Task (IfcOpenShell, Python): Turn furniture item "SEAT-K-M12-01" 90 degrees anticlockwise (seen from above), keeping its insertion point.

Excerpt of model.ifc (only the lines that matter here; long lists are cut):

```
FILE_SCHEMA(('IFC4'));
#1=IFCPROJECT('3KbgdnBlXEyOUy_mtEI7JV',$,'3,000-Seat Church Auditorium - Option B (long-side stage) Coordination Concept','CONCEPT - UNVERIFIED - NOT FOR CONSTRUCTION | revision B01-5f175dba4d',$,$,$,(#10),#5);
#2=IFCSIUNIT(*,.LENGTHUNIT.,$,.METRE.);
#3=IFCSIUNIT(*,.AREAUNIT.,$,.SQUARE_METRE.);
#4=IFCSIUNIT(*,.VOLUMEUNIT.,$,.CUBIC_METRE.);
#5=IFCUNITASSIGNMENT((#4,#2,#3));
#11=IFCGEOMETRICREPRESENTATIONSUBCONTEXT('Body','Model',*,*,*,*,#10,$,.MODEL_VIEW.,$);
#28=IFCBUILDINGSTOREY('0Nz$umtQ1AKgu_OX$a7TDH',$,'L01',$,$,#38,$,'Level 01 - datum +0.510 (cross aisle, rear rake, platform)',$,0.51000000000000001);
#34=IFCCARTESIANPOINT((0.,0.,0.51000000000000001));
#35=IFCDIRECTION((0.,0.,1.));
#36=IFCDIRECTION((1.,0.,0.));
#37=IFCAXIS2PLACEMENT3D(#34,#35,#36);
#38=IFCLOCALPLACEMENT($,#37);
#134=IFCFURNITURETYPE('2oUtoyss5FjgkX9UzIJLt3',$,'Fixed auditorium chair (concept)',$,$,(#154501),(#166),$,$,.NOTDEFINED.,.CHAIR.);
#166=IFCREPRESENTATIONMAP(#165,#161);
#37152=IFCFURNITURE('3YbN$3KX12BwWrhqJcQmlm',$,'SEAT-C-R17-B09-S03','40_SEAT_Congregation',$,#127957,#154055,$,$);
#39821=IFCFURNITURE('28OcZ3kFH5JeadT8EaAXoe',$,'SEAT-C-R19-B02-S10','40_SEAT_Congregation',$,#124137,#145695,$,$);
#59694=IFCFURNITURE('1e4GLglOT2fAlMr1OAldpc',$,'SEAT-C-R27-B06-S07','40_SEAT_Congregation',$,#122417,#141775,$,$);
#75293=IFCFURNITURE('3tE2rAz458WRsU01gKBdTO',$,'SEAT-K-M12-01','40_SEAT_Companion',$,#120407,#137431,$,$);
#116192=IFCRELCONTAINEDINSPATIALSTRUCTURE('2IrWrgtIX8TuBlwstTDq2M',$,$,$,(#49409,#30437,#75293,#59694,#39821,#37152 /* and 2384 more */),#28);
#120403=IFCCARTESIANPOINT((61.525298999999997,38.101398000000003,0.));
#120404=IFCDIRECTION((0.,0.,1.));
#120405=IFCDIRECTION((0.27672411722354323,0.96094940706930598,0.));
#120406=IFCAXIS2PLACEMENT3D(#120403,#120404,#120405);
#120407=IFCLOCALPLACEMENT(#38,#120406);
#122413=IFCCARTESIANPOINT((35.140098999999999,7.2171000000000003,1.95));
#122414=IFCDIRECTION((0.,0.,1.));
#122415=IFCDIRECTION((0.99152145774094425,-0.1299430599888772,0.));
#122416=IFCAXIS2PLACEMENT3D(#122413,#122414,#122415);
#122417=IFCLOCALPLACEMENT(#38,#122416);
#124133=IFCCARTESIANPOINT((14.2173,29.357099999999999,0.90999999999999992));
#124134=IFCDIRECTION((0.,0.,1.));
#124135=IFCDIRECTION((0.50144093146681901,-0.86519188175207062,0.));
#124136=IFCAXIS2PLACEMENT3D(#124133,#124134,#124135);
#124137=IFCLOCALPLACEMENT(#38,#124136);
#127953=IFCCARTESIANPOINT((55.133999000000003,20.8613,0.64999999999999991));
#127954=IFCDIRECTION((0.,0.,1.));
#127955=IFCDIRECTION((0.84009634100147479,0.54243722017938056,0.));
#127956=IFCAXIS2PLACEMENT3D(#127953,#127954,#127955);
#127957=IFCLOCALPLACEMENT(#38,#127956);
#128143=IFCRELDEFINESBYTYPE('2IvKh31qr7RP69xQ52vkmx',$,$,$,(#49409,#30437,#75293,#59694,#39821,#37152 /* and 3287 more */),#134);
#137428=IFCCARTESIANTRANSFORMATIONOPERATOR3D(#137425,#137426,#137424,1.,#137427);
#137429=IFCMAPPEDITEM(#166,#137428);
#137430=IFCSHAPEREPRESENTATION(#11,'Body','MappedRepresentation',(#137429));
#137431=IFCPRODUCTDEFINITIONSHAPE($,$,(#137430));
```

```python
import ifcopenshell
import ifcopenshell.api.geometry
import ifcopenshell.util.placement

model = ifcopenshell.open("model.ifc")

item = model.by_guid("3tE2rAz458WRsU01gKBdTO")
matrix = ifcopenshell.util.placement.get_local_placement(item.ObjectPlacement)
matrix = matrix @ ifcopenshell.util.placement.rotation(90, "Z")
ifcopenshell.api.geometry.edit_object_placement(model, product=item, matrix=matrix, is_si=False)

print(ifcopenshell.util.placement.get_local_placement(item.ObjectPlacement).round(3) + 0.0)

model.write("model_updated.ifc")
```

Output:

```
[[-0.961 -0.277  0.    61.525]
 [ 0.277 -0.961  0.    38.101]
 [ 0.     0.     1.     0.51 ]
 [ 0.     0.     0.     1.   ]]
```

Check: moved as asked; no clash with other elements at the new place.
